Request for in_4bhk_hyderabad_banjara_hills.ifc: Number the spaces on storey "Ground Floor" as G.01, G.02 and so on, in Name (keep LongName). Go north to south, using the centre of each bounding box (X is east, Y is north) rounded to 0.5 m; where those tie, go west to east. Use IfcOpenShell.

First a look at what the model holds.

```python
import ifcopenshell
import ifcopenshell.util.element
import ifcopenshell.util.placement

model = ifcopenshell.open("in_4bhk_hyderabad_banjara_hills.ifc")
print(model.schema)
storey = next(s for s in model.by_type("IfcBuildingStorey") if s.Name == "Ground Floor")
spaces = [e for e in ifcopenshell.util.element.get_decomposition(storey) if e.is_a("IfcSpace")]
for e in sorted(spaces, key=lambda e: e.id()):
    origin = ifcopenshell.util.placement.get_local_placement(e.ObjectPlacement)[:3, 3]
    print(e.id(), e.Name, e.LongName, origin.round(2) + 0.0, sep=" | ")
```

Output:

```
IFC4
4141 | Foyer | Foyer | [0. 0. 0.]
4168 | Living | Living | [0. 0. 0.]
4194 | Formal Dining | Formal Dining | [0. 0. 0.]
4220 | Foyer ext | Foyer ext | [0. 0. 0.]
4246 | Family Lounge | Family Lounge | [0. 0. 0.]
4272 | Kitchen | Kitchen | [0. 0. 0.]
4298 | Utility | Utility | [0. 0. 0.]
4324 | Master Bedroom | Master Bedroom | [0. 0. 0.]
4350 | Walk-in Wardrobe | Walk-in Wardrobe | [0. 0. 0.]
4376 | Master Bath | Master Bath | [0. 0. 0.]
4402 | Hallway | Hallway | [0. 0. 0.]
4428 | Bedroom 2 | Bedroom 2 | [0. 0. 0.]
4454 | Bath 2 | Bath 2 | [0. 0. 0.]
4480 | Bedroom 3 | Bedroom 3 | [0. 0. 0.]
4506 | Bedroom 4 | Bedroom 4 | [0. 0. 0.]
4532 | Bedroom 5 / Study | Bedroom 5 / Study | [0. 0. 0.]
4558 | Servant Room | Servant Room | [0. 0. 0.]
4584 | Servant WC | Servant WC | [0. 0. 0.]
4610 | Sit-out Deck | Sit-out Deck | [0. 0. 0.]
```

```python
import ifcopenshell
import ifcopenshell.geom
import ifcopenshell.util.element
import ifcopenshell.util.shape

model = ifcopenshell.open("in_4bhk_hyderabad_banjara_hills.ifc")
settings = ifcopenshell.geom.settings()
settings.set("use-world-coords", True)


def centre(element):
    shape = ifcopenshell.geom.create_shape(settings, element)
    return ifcopenshell.util.shape.get_bbox_centroid(shape.geometry)


storey = next(s for s in model.by_type("IfcBuildingStorey") if s.Name == "Ground Floor")
spaces = [e for e in ifcopenshell.util.element.get_decomposition(storey) if e.is_a("IfcSpace")]

# Insertion points can sit at a corner or the storey origin, so sort by the geometry (in metres).
centres = {e: centre(e) for e in spaces}
spaces.sort(key=lambda e: (-round(centres[e][1] / 0.5), centres[e][0]))

for i, e in enumerate(spaces, start=1):
    number = f"G.{i:02d}"
    e.Name = number
    print(e.id(), number)

model.write("in_4bhk_hyderabad_banjara_hills-out.ifc")
```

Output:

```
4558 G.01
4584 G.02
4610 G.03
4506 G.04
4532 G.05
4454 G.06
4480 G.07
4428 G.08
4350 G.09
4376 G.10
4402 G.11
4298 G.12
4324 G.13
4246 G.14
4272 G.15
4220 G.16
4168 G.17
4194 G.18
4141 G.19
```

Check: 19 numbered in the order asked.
